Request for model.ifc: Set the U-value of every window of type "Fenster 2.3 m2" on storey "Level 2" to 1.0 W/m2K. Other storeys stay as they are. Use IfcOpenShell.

First a look at what the model holds.

```python
import ifcopenshell
import ifcopenshell.util.element

model = ifcopenshell.open("model.ifc")
print(model.schema)
storey = next(s for s in model.by_type("IfcBuildingStorey") if s.Name == "Level 2")
windows = [e for e in ifcopenshell.util.element.get_decomposition(storey) if e.is_a("IfcWindow")]
seen = {}
for e in windows:
    element_type = ifcopenshell.util.element.get_type(e)
    key = (element_type.Name if element_type != e and element_type else None, ifcopenshell.util.element.get_pset(e, "Pset_WindowCommon", "ThermalTransmittance"))
    seen[key] = seen.get(key, 0) + 1
for (name, value), count in sorted(seen.items(), key=str):
    print(count, "x", name, "|", value)
```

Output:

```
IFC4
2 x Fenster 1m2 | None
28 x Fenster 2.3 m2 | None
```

```python
import ifcopenshell
import ifcopenshell.api.pset
import ifcopenshell.util.element

model = ifcopenshell.open("model.ifc")

storey = next(s for s in model.by_type("IfcBuildingStorey") if s.Name == "Level 2")
windows = [e for e in ifcopenshell.util.element.get_decomposition(storey) if e.is_a("IfcWindow")]

count = 0
for e in windows:
    element_type = ifcopenshell.util.element.get_type(e)
    if element_type in (None, e) or element_type.Name != "Fenster 2.3 m2":
        continue
    # add_pset returns the element's existing set when there is one.
    pset = ifcopenshell.api.pset.add_pset(model, product=e, name="Pset_WindowCommon")
    ifcopenshell.api.pset.edit_pset(model, pset=pset, properties={"ThermalTransmittance": 1.0})
    count += 1

print(count, "windows updated")

model.write("model_v2.ifc")
```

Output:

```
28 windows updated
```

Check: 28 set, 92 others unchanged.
